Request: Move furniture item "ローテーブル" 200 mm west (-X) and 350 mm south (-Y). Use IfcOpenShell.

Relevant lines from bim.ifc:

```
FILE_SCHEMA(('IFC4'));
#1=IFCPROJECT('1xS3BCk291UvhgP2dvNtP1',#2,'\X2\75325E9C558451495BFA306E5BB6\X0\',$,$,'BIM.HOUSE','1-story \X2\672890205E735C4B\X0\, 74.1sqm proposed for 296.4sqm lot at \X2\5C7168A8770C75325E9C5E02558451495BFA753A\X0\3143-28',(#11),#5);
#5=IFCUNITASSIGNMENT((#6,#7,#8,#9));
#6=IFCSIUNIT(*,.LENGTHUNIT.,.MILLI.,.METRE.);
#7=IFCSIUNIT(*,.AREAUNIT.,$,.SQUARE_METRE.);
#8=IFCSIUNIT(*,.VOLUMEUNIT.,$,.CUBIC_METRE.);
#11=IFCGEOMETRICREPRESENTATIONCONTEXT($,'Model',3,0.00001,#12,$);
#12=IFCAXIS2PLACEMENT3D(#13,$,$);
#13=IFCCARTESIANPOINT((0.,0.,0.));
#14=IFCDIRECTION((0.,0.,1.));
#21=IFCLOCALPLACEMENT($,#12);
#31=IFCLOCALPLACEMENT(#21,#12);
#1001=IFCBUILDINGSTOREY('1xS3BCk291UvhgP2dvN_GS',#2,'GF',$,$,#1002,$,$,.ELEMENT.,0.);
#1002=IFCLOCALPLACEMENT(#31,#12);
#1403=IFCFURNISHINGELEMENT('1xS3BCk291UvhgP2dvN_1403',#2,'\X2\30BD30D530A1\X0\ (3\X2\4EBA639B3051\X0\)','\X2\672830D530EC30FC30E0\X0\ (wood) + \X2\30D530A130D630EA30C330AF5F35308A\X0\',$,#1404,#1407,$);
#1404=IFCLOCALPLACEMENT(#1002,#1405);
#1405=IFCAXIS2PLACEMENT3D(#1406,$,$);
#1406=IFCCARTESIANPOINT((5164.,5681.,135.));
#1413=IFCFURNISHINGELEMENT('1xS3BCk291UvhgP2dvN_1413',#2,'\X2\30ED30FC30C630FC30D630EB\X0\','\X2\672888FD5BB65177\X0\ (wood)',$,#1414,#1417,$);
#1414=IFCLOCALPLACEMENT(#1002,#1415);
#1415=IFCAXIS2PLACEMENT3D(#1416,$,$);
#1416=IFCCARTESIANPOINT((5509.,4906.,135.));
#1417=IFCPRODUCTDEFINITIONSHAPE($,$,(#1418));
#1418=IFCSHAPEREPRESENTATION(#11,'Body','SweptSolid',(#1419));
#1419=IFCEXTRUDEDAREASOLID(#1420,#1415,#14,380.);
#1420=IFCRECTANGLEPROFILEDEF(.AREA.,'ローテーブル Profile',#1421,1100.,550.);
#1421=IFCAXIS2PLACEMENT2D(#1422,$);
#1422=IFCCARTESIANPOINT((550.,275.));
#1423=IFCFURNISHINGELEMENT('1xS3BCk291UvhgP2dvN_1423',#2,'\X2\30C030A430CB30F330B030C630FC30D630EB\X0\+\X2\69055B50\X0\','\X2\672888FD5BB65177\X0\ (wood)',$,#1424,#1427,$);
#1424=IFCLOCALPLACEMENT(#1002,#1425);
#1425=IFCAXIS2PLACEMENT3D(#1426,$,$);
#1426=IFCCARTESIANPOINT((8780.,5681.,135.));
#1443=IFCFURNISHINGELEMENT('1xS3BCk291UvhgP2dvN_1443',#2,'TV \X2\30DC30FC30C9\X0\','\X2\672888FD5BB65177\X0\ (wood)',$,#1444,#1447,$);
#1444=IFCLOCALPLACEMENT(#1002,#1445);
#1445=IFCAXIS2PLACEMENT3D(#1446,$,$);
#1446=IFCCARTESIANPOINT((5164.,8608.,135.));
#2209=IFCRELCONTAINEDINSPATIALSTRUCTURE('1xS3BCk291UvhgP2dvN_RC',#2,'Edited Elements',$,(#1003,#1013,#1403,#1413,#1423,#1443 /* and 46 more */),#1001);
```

```python
import ifcopenshell
import ifcopenshell.api.geometry
import ifcopenshell.util.placement

model = ifcopenshell.open("bim.ifc")

item = model.by_guid("1xS3BCk291UvhgP2dvN_1413")
matrix = ifcopenshell.util.placement.get_local_placement(item.ObjectPlacement)
matrix[0, 3] -= 200.0
matrix[1, 3] -= 350.0
ifcopenshell.api.geometry.edit_object_placement(model, product=item, matrix=matrix, is_si=False)

print(ifcopenshell.util.placement.get_local_placement(item.ObjectPlacement).round(3) + 0.0)

model.write("bim-out.ifc")
```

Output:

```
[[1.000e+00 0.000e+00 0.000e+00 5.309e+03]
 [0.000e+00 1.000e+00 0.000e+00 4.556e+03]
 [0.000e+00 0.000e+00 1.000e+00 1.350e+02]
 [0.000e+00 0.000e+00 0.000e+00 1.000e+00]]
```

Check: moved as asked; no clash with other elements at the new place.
